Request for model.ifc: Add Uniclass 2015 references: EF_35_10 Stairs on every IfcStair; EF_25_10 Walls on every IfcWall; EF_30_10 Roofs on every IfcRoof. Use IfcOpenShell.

First a look at what the model holds.

```python
import ifcopenshell

model = ifcopenshell.open("model.ifc")
print(model.schema)
print("classifications:", [c.Name for c in model.by_type("IfcClassification")])
for ifc_class in ("IfcDoor", "IfcRoof", "IfcStair", "IfcWall", "IfcWindow"):
    print(ifc_class, len(model.by_type(ifc_class)))
```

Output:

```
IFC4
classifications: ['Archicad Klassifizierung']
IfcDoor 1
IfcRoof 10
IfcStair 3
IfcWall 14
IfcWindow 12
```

```python
import ifcopenshell
import ifcopenshell.api.classification

model = ifcopenshell.open("model.ifc")

system = ifcopenshell.api.classification.add_classification(model, classification="Uniclass 2015")

codes = {
    "IfcStair": ("EF_35_10", "Stairs"),
    "IfcWall": ("EF_25_10", "Walls"),
    "IfcRoof": ("EF_30_10", "Roofs"),
}
for ifc_class, (code, name) in codes.items():
    products = model.by_type(ifc_class)
    ifcopenshell.api.classification.add_reference(
        model, products=products, classification=system, identification=code, name=name
    )
    print(code, len(products))

model.write("model_updated.ifc")
```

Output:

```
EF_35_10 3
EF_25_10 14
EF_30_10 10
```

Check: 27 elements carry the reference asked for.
